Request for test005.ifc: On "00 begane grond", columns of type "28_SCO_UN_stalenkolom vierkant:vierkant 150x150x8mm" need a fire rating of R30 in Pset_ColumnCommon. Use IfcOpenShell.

First a look at what the model holds.

```python
import ifcopenshell
import ifcopenshell.util.element

model = ifcopenshell.open("test005.ifc")
print(model.schema)
storey = next(s for s in model.by_type("IfcBuildingStorey") if s.Name == "00 begane grond")
columns = [e for e in ifcopenshell.util.element.get_decomposition(storey) if e.is_a("IfcColumn")]
seen = {}
for e in columns:
    element_type = ifcopenshell.util.element.get_type(e)
    key = (element_type.Name if element_type != e and element_type else None, ifcopenshell.util.element.get_pset(e, "Pset_ColumnCommon", "FireRating"))
    seen[key] = seen.get(key, 0) + 1
for (name, value), count in sorted(seen.items(), key=str):
    print(count, "x", name, "|", value)
```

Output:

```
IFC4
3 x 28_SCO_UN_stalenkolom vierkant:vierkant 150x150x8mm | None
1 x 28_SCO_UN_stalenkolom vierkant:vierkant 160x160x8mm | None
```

```python
import ifcopenshell
import ifcopenshell.api.pset
import ifcopenshell.util.element

model = ifcopenshell.open("test005.ifc")

storey = next(s for s in model.by_type("IfcBuildingStorey") if s.Name == "00 begane grond")
columns = [e for e in ifcopenshell.util.element.get_decomposition(storey) if e.is_a("IfcColumn")]

count = 0
for e in columns:
    element_type = ifcopenshell.util.element.get_type(e)
    if element_type in (None, e) or element_type.Name != "28_SCO_UN_stalenkolom vierkant:vierkant 150x150x8mm":
        continue
    # add_pset returns the element's existing set when there is one.
    pset = ifcopenshell.api.pset.add_pset(model, product=e, name="Pset_ColumnCommon")
    ifcopenshell.api.pset.edit_pset(model, pset=pset, properties={"FireRating": "R30"})
    count += 1

print(count, "columns updated")

model.write("test005_edited.ifc")
```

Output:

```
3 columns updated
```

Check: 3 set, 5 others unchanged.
